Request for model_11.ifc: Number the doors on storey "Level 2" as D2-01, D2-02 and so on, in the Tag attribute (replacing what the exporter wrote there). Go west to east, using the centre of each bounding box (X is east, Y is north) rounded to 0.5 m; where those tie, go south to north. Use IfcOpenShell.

First a look at what the model holds.

```python
import ifcopenshell
import ifcopenshell.util.element
import ifcopenshell.util.placement

model = ifcopenshell.open("model_11.ifc")
print(model.schema)
storey = next(s for s in model.by_type("IfcBuildingStorey") if s.Name == "Level 2")
doors = [e for e in ifcopenshell.util.element.get_decomposition(storey) if e.is_a("IfcDoor")]
for e in sorted(doors, key=lambda e: e.id()):
    origin = ifcopenshell.util.placement.get_local_placement(e.ObjectPlacement)[:3, 3]
    print(e.id(), e.Tag, e.Name, origin.round(2) + 0.0, sep=" | ")
```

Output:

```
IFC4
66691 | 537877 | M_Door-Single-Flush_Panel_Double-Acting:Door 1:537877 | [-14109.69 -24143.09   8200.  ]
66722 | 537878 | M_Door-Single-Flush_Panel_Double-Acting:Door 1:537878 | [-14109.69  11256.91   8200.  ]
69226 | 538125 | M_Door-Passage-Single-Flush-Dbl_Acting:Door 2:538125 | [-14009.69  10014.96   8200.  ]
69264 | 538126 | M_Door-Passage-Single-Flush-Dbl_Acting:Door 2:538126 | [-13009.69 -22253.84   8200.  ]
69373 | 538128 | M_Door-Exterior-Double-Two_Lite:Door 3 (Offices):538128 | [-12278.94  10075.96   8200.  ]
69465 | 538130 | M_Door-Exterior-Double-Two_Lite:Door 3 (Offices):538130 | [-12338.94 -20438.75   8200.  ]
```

```python
import ifcopenshell
import ifcopenshell.geom
import ifcopenshell.util.element
import ifcopenshell.util.shape

model = ifcopenshell.open("model_11.ifc")
settings = ifcopenshell.geom.settings()
settings.set("use-world-coords", True)


def centre(element):
    shape = ifcopenshell.geom.create_shape(settings, element)
    return ifcopenshell.util.shape.get_bbox_centroid(shape.geometry)


storey = next(s for s in model.by_type("IfcBuildingStorey") if s.Name == "Level 2")
doors = [e for e in ifcopenshell.util.element.get_decomposition(storey) if e.is_a("IfcDoor")]

# Insertion points can sit at a corner or the storey origin, so sort by the geometry (in metres).
centres = {e: centre(e) for e in doors}
doors.sort(key=lambda e: (round(centres[e][0] / 0.5), centres[e][1]))

for i, e in enumerate(doors, start=1):
    number = f"D2-{i:02d}"
    e.Tag = number
    print(e.id(), number)

model.write("model_11-out.ifc")
```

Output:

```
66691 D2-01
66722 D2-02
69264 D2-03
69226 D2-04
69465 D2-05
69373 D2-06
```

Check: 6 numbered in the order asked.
